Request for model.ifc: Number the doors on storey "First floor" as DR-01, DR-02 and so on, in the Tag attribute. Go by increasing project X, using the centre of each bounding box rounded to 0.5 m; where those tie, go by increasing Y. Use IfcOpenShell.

First a look at what the model holds.

```python
import ifcopenshell
import ifcopenshell.util.element
import ifcopenshell.util.placement

model = ifcopenshell.open("model.ifc")
print(model.schema)
storey = next(s for s in model.by_type("IfcBuildingStorey") if s.Name == "First floor")
doors = [e for e in ifcopenshell.util.element.get_decomposition(storey) if e.is_a("IfcDoor")]
for e in sorted(doors, key=lambda e: e.id()):
    origin = ifcopenshell.util.placement.get_local_placement(e.ObjectPlacement)[:3, 3]
    print(e.id(), e.Tag, e.Name, origin.round(2) + 0.0, sep=" | ")
```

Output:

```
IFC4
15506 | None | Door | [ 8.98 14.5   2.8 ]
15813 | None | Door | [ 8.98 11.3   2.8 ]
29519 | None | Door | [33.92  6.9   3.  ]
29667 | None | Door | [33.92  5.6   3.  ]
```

```python
import ifcopenshell
import ifcopenshell.geom
import ifcopenshell.util.element
import ifcopenshell.util.shape

model = ifcopenshell.open("model.ifc")
settings = ifcopenshell.geom.settings()
settings.set("use-world-coords", True)


def centre(element):
    shape = ifcopenshell.geom.create_shape(settings, element)
    return ifcopenshell.util.shape.get_bbox_centroid(shape.geometry)


storey = next(s for s in model.by_type("IfcBuildingStorey") if s.Name == "First floor")
doors = [e for e in ifcopenshell.util.element.get_decomposition(storey) if e.is_a("IfcDoor")]

# Insertion points can sit at a corner or the storey origin, so sort by the geometry (in metres).
centres = {e: centre(e) for e in doors}
doors.sort(key=lambda e: (round(centres[e][0] / 0.5), centres[e][1]))

for i, e in enumerate(doors, start=1):
    number = f"DR-{i:02d}"
    e.Tag = number
    print(e.id(), number)

model.write("model_rev.ifc")
```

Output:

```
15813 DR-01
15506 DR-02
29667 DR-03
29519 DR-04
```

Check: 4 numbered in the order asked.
